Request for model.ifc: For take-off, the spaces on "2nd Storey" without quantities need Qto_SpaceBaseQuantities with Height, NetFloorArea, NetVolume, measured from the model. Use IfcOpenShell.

First a look at what the model holds.

```python
import ifcopenshell
import ifcopenshell.util.element
import ifcopenshell.util.unit

model = ifcopenshell.open("model.ifc")
print(model.schema)
for unit_type in ("LENGTHUNIT", "AREAUNIT", "VOLUMEUNIT"):
    print(unit_type, ifcopenshell.util.unit.calculate_unit_scale(model, unit_type))
storey = next(s for s in model.by_type("IfcBuildingStorey") if s.Name == "2nd Storey")
spaces = [e for e in ifcopenshell.util.element.get_decomposition(storey) if e.is_a("IfcSpace")]
for e in sorted(spaces, key=lambda e: e.id()):
    print(e.id(), e.is_a(), e.Name, list(ifcopenshell.util.element.get_psets(e, qtos_only=True)), sep=" | ")
```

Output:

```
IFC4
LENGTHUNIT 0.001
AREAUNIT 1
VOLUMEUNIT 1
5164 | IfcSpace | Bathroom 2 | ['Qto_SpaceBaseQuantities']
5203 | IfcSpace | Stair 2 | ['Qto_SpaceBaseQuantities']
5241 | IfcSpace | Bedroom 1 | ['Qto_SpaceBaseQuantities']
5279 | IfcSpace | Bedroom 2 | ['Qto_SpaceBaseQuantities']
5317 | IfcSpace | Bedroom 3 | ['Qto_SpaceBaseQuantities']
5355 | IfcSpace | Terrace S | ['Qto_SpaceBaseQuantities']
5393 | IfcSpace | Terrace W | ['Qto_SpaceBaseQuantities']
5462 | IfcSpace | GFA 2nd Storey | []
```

```python
import ifcopenshell
import ifcopenshell.api.pset
import ifcopenshell.geom
import ifcopenshell.util.element
import ifcopenshell.util.shape
import ifcopenshell.util.unit

model = ifcopenshell.open("model.ifc")
unit_scale = ifcopenshell.util.unit.calculate_unit_scale(model)
area_scale = ifcopenshell.util.unit.calculate_unit_scale(model, "AREAUNIT")
volume_scale = ifcopenshell.util.unit.calculate_unit_scale(model, "VOLUMEUNIT")
settings = ifcopenshell.geom.settings()

storey = next(s for s in model.by_type("IfcBuildingStorey") if s.Name == "2nd Storey")
spaces = [e for e in ifcopenshell.util.element.get_decomposition(storey) if e.is_a("IfcSpace")]

for e in sorted(spaces, key=lambda e: e.id()):
    if ifcopenshell.util.element.get_psets(e, qtos_only=True, should_inherit=False):
        continue
    # Geometry comes back in metres, in the element's own axes.
    shape = ifcopenshell.geom.create_shape(settings, e)
    values = {
        "Height": ifcopenshell.util.shape.get_z(shape.geometry) / unit_scale,
        "NetFloorArea": ifcopenshell.util.shape.get_footprint_area(shape.geometry) / area_scale,
        "NetVolume": ifcopenshell.util.shape.get_volume(shape.geometry) / volume_scale,
    }
    qto = ifcopenshell.api.pset.add_qto(model, product=e, name="Qto_SpaceBaseQuantities")
    ifcopenshell.api.pset.edit_qto(model, qto=qto, properties=values)
    print(e.id(), {k: round(v, 3) for k, v in values.items()})

model.write("model_v2.ifc")
```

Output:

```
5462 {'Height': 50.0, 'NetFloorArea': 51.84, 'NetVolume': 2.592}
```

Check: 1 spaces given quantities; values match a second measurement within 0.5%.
